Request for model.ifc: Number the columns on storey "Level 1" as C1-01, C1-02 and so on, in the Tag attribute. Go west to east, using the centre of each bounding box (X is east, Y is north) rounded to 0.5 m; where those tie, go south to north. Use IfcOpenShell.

First a look at what the model holds.

```python
import ifcopenshell
import ifcopenshell.util.element
import ifcopenshell.util.placement

model = ifcopenshell.open("model.ifc")
print(model.schema)
storey = next(s for s in model.by_type("IfcBuildingStorey") if s.Name == "Level 1")
columns = [e for e in ifcopenshell.util.element.get_decomposition(storey) if e.is_a("IfcColumn")]
for e in sorted(columns, key=lambda e: e.id()):
    origin = ifcopenshell.util.placement.get_local_placement(e.ObjectPlacement)[:3, 3]
    print(e.id(), e.Tag, e.Name, origin.round(2) + 0.0, sep=" | ")
```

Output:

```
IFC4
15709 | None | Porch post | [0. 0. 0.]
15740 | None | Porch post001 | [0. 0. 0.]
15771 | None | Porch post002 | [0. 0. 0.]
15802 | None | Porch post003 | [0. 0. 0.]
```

```python
import ifcopenshell
import ifcopenshell.geom
import ifcopenshell.util.element
import ifcopenshell.util.shape

model = ifcopenshell.open("model.ifc")
settings = ifcopenshell.geom.settings()
settings.set("use-world-coords", True)


def centre(element):
    shape = ifcopenshell.geom.create_shape(settings, element)
    return ifcopenshell.util.shape.get_bbox_centroid(shape.geometry)


storey = next(s for s in model.by_type("IfcBuildingStorey") if s.Name == "Level 1")
columns = [e for e in ifcopenshell.util.element.get_decomposition(storey) if e.is_a("IfcColumn")]

# Insertion points can sit at a corner or the storey origin, so sort by the geometry (in metres).
centres = {e: centre(e) for e in columns}
columns.sort(key=lambda e: (round(centres[e][0] / 0.5), centres[e][1]))

for i, e in enumerate(columns, start=1):
    number = f"C1-{i:02d}"
    e.Tag = number
    print(e.id(), number)

model.write("model_edited.ifc")
```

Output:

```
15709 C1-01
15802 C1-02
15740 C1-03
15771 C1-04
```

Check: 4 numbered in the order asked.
